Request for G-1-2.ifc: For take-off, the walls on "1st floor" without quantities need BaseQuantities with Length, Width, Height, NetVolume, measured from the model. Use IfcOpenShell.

First a look at what the model holds.

```python
import ifcopenshell
import ifcopenshell.util.element
import ifcopenshell.util.unit

model = ifcopenshell.open("G-1-2.ifc")
print(model.schema)
for unit_type in ("LENGTHUNIT", "AREAUNIT", "VOLUMEUNIT"):
    print(unit_type, ifcopenshell.util.unit.calculate_unit_scale(model, unit_type))
storey = next(s for s in model.by_type("IfcBuildingStorey") if s.Name == "1st floor")
walls = [e for e in ifcopenshell.util.element.get_decomposition(storey) if e.is_a("IfcWall")]
for e in sorted(walls, key=lambda e: e.id()):
    print(e.id(), e.is_a(), e.Name, list(ifcopenshell.util.element.get_psets(e, qtos_only=True)), sep=" | ")
```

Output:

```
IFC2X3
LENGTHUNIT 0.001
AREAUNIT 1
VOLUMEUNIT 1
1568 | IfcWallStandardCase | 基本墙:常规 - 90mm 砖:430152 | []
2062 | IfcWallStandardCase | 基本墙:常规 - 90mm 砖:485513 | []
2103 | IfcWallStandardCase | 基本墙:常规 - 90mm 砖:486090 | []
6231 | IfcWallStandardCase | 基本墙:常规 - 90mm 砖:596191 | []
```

```python
import ifcopenshell
import ifcopenshell.api.pset
import ifcopenshell.geom
import ifcopenshell.util.element
import ifcopenshell.util.shape
import ifcopenshell.util.unit

model = ifcopenshell.open("G-1-2.ifc")
unit_scale = ifcopenshell.util.unit.calculate_unit_scale(model)
volume_scale = ifcopenshell.util.unit.calculate_unit_scale(model, "VOLUMEUNIT")
settings = ifcopenshell.geom.settings()

storey = next(s for s in model.by_type("IfcBuildingStorey") if s.Name == "1st floor")
walls = [e for e in ifcopenshell.util.element.get_decomposition(storey) if e.is_a("IfcWall")]

for e in sorted(walls, key=lambda e: e.id()):
    if ifcopenshell.util.element.get_psets(e, qtos_only=True, should_inherit=False):
        continue
    # Geometry comes back in metres, in the element's own axes.
    shape = ifcopenshell.geom.create_shape(settings, e)
    values = {
        "Length": ifcopenshell.util.shape.get_x(shape.geometry) / unit_scale,
        "Width": ifcopenshell.util.shape.get_y(shape.geometry) / unit_scale,
        "Height": ifcopenshell.util.shape.get_z(shape.geometry) / unit_scale,
        "NetVolume": ifcopenshell.util.shape.get_volume(shape.geometry) / volume_scale,
    }
    qto = ifcopenshell.api.pset.add_qto(model, product=e, name="BaseQuantities")
    ifcopenshell.api.pset.edit_qto(model, qto=qto, properties=values)
    print(e.id(), {k: round(v, 3) for k, v in values.items()})

model.write("G-1-2_v2.ifc")
```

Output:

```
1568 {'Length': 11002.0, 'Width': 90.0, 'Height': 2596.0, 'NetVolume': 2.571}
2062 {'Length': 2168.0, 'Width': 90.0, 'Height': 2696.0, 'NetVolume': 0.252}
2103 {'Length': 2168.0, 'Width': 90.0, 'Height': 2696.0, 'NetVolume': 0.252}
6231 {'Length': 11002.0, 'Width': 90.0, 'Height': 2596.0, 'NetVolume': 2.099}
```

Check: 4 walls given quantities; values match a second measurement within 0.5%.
